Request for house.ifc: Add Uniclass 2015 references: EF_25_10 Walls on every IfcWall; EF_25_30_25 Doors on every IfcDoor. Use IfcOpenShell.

First a look at what the model holds.

```python
import ifcopenshell

model = ifcopenshell.open("house.ifc")
print(model.schema)
print("classifications:", [c.Name for c in model.by_type("IfcClassification")])
for ifc_class in ("IfcDoor", "IfcRoof", "IfcStair", "IfcWall", "IfcWindow"):
    print(ifc_class, len(model.by_type(ifc_class)))
```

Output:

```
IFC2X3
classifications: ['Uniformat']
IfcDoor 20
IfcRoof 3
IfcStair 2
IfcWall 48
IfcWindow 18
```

```python
import ifcopenshell
import ifcopenshell.api.classification

model = ifcopenshell.open("house.ifc")

# IFC2X3 requires Source and Edition and has no link from the project to the system.
system = model.create_entity("IfcClassification", Source="NBS", Edition="2015", Name="Uniclass 2015")

codes = {
    "IfcWall": ("EF_25_10", "Walls"),
    "IfcDoor": ("EF_25_30_25", "Doors"),
}
for ifc_class, (code, name) in codes.items():
    products = model.by_type(ifc_class)
    ifcopenshell.api.classification.add_reference(
        model, products=products, classification=system, identification=code, name=name
    )
    print(code, len(products))

model.write("house_updated.ifc")
```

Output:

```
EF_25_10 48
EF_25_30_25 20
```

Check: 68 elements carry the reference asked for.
